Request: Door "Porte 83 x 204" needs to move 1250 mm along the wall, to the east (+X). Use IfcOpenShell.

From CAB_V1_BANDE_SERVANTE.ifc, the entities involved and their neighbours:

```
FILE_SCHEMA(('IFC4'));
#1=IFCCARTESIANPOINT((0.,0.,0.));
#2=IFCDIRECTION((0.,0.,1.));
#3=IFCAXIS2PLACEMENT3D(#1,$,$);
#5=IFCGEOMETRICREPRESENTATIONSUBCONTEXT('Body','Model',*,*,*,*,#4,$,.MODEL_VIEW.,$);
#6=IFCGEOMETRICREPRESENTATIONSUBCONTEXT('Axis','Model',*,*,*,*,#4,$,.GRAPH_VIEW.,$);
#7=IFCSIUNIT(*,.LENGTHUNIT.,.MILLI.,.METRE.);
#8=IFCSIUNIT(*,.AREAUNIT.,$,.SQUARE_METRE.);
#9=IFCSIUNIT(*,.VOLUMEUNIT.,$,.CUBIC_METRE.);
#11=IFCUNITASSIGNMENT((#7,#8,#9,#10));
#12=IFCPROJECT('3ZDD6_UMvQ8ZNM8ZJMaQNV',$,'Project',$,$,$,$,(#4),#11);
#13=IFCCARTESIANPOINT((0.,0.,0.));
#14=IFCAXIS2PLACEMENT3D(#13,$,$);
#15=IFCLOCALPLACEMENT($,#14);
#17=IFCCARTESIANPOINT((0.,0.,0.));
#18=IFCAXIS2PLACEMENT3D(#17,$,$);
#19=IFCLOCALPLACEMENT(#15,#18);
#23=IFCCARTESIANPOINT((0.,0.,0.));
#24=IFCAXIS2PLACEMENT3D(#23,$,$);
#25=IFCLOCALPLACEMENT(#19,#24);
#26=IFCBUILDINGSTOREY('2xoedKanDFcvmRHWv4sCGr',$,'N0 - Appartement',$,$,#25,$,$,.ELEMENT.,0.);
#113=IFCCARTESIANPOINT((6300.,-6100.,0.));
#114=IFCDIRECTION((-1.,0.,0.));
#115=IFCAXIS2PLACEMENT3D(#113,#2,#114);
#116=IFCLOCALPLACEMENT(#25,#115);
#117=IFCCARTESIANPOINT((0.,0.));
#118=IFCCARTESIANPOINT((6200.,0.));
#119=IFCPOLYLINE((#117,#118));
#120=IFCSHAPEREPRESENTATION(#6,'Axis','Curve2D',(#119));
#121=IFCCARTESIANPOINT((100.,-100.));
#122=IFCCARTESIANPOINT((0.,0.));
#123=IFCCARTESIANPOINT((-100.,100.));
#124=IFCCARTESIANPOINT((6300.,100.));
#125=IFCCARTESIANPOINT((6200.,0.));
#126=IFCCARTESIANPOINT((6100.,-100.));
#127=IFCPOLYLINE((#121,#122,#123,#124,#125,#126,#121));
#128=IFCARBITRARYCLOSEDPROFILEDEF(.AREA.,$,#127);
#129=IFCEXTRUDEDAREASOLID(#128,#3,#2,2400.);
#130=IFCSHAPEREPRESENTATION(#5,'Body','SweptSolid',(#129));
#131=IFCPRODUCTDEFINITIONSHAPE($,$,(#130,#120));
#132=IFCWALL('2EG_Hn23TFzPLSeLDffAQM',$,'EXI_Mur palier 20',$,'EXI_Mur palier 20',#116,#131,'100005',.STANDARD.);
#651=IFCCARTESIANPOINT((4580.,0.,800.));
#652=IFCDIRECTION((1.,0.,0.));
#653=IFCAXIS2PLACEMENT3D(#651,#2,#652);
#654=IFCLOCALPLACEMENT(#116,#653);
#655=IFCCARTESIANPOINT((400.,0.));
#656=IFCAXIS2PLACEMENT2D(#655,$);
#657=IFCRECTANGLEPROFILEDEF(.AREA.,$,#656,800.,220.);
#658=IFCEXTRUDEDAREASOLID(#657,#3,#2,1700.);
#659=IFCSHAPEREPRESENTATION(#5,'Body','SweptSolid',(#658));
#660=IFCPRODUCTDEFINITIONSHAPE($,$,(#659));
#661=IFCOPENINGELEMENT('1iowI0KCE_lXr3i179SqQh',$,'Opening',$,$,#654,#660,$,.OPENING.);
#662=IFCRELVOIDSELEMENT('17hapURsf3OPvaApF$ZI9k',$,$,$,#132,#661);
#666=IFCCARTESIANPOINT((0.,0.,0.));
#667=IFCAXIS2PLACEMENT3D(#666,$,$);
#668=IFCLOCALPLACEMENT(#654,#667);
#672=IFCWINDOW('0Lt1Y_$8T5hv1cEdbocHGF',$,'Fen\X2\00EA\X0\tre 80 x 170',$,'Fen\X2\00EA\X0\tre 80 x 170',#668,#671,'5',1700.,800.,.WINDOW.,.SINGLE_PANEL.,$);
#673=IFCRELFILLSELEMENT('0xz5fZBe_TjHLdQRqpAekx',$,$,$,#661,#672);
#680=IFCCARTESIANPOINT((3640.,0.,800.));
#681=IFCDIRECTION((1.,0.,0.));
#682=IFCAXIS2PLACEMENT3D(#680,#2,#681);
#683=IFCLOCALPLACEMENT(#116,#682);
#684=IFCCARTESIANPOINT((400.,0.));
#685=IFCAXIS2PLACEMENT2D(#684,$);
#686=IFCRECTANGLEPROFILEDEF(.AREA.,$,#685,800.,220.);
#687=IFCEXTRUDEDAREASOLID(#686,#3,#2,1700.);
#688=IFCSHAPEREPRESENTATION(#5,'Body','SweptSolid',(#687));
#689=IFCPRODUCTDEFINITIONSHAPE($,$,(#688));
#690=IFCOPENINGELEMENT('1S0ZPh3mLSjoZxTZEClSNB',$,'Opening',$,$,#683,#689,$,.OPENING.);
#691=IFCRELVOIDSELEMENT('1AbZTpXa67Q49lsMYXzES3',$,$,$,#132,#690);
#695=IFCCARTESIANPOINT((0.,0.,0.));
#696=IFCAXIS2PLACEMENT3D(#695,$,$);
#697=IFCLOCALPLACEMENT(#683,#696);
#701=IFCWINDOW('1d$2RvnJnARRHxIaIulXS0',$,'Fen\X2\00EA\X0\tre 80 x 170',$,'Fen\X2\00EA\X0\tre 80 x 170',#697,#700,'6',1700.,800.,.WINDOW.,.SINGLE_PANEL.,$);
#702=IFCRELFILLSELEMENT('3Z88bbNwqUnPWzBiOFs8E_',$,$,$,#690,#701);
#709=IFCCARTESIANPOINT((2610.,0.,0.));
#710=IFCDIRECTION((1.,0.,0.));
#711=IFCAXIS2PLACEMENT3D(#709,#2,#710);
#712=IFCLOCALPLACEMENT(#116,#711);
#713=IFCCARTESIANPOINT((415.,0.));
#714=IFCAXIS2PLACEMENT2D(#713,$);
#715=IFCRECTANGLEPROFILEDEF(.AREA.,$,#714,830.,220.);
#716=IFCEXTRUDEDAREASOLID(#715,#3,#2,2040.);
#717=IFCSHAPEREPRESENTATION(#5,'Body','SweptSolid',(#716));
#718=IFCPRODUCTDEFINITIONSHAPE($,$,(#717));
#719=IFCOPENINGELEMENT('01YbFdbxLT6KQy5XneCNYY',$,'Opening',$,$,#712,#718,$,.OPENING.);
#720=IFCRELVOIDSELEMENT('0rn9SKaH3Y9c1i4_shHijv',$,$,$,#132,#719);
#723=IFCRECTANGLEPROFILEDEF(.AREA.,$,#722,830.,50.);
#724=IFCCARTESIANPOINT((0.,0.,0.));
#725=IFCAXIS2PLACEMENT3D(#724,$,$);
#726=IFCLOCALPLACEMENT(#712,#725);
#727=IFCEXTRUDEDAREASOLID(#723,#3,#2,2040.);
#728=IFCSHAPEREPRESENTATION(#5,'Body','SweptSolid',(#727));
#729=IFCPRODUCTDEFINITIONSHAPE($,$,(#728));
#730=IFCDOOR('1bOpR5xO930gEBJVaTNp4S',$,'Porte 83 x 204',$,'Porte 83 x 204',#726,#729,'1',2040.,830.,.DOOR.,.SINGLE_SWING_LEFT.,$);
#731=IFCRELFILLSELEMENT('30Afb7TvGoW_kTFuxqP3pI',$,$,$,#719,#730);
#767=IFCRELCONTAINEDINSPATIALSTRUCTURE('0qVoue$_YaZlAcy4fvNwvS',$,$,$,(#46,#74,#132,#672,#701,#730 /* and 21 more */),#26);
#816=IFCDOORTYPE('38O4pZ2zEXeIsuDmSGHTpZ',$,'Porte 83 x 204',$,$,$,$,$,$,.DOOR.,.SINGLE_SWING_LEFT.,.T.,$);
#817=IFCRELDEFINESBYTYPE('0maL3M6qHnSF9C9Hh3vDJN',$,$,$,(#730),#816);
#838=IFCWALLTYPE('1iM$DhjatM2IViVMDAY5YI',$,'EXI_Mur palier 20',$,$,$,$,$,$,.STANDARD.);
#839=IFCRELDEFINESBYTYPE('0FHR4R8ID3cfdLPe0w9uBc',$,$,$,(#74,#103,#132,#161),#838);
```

```python
import ifcopenshell
import ifcopenshell.api.geometry
import ifcopenshell.util.placement

model = ifcopenshell.open("CAB_V1_BANDE_SERVANTE.ifc")

door = model.by_guid("1bOpR5xO930gEBJVaTNp4S")
opening = door.FillsVoids[0].RelatingOpeningElement
wall = opening.VoidsElements[0].RelatingBuildingElement

wall_matrix = ifcopenshell.util.placement.get_local_placement(wall.ObjectPlacement)
shift = wall_matrix[:3, 0] * -1250.0
before = ifcopenshell.util.placement.get_local_placement(door.ObjectPlacement)[:3, 3].copy()

# The door is placed relative to its opening, so it follows when the opening moves.
matrix = ifcopenshell.util.placement.get_local_placement(opening.ObjectPlacement)
matrix[:3, 3] += shift
ifcopenshell.api.geometry.edit_object_placement(
    model, product=opening, matrix=matrix, is_si=False, should_transform_children=True
)

after = ifcopenshell.util.placement.get_local_placement(door.ObjectPlacement)[:3, 3]
print("door moved by", (after - before).round(3) + 0.0)

model.write("CAB_V1_BANDE_SERVANTE_rev.ifc")
```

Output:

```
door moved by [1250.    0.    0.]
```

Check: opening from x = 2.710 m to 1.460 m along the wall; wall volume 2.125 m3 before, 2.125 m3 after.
